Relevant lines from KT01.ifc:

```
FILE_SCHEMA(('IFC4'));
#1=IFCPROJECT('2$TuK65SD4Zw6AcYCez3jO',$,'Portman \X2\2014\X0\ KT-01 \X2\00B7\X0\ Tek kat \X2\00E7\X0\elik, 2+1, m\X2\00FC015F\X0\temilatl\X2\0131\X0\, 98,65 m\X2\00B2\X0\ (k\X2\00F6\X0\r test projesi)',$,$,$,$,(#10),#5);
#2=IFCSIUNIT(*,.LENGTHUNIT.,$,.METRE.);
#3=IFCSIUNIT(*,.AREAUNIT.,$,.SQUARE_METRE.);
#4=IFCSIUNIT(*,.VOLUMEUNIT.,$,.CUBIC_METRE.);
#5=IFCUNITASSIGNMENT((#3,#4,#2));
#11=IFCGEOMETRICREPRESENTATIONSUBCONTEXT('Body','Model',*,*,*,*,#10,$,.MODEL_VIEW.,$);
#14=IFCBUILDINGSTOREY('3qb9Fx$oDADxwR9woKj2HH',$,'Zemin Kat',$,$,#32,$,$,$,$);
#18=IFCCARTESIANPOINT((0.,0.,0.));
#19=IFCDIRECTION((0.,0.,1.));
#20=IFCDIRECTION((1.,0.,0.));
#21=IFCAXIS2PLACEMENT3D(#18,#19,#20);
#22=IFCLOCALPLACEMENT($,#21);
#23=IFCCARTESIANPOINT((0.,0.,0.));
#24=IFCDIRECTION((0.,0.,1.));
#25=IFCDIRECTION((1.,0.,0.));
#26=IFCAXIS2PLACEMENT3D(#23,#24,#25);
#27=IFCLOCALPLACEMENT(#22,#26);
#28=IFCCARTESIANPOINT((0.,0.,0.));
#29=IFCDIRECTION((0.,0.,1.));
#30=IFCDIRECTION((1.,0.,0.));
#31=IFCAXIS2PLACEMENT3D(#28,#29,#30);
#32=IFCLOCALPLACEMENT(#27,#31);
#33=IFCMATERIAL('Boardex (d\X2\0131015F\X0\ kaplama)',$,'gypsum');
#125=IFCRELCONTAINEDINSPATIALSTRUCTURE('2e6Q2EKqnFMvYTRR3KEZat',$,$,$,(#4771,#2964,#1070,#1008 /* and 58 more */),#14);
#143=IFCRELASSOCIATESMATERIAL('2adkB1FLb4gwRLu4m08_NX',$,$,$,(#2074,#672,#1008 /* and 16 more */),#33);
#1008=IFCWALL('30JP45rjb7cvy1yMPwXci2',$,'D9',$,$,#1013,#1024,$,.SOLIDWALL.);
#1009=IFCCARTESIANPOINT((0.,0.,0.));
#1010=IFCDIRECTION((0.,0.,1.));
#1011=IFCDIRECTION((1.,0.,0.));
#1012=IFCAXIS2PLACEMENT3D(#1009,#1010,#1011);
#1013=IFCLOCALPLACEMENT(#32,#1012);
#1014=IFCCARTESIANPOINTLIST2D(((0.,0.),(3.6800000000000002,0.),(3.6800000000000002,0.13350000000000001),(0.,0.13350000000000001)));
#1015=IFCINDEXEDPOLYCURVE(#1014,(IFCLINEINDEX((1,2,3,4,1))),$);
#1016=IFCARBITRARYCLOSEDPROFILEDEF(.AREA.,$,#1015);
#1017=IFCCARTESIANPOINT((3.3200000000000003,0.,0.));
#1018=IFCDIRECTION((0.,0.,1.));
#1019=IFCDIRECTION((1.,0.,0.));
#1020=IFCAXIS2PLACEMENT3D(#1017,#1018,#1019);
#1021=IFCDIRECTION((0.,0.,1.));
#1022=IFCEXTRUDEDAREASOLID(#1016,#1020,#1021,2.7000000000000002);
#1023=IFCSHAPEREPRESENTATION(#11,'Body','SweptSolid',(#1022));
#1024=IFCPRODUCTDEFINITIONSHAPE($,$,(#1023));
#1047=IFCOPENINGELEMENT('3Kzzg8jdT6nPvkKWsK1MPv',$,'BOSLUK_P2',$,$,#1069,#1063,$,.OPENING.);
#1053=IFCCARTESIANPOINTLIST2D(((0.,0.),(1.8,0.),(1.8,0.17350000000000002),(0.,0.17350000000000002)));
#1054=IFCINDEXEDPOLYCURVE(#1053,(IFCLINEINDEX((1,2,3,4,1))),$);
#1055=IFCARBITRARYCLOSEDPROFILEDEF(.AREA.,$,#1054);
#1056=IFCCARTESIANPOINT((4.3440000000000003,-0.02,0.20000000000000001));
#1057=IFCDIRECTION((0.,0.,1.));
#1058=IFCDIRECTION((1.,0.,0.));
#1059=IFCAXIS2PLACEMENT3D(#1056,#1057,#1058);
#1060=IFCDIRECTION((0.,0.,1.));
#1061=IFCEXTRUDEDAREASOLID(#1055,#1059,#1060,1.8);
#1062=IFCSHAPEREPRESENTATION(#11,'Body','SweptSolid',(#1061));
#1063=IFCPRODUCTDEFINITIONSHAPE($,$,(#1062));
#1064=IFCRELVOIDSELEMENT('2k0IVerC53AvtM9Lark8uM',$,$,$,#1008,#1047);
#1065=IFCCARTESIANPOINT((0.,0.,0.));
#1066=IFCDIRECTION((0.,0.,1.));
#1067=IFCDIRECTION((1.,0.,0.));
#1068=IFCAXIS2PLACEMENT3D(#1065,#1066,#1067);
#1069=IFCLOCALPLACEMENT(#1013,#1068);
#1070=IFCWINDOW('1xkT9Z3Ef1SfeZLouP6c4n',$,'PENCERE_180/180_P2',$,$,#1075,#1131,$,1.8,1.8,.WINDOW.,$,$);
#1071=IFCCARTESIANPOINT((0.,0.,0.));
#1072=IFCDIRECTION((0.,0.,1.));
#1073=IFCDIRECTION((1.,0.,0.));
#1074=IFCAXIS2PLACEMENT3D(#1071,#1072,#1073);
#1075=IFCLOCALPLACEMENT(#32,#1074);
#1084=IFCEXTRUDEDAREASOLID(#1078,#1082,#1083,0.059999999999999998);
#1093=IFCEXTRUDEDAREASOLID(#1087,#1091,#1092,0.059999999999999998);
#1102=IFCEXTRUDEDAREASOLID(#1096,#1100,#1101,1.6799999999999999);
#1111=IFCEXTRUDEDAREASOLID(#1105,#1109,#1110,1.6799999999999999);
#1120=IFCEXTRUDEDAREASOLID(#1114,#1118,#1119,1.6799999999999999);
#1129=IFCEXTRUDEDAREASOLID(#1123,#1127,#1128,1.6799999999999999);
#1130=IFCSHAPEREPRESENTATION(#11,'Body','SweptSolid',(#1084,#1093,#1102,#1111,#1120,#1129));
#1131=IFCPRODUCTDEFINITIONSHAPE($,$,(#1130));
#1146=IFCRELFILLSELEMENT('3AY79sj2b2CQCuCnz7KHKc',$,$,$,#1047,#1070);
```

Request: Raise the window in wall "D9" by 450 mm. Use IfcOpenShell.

```python
import numpy as np
import ifcopenshell
import ifcopenshell.api.geometry
import ifcopenshell.util.placement
import ifcopenshell.util.unit

model = ifcopenshell.open("KT01.ifc")
unit_scale = ifcopenshell.util.unit.calculate_unit_scale(model)

window = model.by_id(1070)
opening = window.FillsVoids[0].RelatingOpeningElement
dz = 0.45

shift = np.array([0.0, 0.0, dz])
# The window is not placed relative to its opening, so move both.
for product in (opening, window):
    matrix = ifcopenshell.util.placement.get_local_placement(product.ObjectPlacement)
    matrix[:3, 3] += shift
    ifcopenshell.api.geometry.edit_object_placement(model, product=product, matrix=matrix, is_si=False)

print(f"moved by {dz * unit_scale:+.3f} m")

model.write("KT01_updated.ifc")
```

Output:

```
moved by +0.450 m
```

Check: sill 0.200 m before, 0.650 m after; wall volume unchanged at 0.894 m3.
